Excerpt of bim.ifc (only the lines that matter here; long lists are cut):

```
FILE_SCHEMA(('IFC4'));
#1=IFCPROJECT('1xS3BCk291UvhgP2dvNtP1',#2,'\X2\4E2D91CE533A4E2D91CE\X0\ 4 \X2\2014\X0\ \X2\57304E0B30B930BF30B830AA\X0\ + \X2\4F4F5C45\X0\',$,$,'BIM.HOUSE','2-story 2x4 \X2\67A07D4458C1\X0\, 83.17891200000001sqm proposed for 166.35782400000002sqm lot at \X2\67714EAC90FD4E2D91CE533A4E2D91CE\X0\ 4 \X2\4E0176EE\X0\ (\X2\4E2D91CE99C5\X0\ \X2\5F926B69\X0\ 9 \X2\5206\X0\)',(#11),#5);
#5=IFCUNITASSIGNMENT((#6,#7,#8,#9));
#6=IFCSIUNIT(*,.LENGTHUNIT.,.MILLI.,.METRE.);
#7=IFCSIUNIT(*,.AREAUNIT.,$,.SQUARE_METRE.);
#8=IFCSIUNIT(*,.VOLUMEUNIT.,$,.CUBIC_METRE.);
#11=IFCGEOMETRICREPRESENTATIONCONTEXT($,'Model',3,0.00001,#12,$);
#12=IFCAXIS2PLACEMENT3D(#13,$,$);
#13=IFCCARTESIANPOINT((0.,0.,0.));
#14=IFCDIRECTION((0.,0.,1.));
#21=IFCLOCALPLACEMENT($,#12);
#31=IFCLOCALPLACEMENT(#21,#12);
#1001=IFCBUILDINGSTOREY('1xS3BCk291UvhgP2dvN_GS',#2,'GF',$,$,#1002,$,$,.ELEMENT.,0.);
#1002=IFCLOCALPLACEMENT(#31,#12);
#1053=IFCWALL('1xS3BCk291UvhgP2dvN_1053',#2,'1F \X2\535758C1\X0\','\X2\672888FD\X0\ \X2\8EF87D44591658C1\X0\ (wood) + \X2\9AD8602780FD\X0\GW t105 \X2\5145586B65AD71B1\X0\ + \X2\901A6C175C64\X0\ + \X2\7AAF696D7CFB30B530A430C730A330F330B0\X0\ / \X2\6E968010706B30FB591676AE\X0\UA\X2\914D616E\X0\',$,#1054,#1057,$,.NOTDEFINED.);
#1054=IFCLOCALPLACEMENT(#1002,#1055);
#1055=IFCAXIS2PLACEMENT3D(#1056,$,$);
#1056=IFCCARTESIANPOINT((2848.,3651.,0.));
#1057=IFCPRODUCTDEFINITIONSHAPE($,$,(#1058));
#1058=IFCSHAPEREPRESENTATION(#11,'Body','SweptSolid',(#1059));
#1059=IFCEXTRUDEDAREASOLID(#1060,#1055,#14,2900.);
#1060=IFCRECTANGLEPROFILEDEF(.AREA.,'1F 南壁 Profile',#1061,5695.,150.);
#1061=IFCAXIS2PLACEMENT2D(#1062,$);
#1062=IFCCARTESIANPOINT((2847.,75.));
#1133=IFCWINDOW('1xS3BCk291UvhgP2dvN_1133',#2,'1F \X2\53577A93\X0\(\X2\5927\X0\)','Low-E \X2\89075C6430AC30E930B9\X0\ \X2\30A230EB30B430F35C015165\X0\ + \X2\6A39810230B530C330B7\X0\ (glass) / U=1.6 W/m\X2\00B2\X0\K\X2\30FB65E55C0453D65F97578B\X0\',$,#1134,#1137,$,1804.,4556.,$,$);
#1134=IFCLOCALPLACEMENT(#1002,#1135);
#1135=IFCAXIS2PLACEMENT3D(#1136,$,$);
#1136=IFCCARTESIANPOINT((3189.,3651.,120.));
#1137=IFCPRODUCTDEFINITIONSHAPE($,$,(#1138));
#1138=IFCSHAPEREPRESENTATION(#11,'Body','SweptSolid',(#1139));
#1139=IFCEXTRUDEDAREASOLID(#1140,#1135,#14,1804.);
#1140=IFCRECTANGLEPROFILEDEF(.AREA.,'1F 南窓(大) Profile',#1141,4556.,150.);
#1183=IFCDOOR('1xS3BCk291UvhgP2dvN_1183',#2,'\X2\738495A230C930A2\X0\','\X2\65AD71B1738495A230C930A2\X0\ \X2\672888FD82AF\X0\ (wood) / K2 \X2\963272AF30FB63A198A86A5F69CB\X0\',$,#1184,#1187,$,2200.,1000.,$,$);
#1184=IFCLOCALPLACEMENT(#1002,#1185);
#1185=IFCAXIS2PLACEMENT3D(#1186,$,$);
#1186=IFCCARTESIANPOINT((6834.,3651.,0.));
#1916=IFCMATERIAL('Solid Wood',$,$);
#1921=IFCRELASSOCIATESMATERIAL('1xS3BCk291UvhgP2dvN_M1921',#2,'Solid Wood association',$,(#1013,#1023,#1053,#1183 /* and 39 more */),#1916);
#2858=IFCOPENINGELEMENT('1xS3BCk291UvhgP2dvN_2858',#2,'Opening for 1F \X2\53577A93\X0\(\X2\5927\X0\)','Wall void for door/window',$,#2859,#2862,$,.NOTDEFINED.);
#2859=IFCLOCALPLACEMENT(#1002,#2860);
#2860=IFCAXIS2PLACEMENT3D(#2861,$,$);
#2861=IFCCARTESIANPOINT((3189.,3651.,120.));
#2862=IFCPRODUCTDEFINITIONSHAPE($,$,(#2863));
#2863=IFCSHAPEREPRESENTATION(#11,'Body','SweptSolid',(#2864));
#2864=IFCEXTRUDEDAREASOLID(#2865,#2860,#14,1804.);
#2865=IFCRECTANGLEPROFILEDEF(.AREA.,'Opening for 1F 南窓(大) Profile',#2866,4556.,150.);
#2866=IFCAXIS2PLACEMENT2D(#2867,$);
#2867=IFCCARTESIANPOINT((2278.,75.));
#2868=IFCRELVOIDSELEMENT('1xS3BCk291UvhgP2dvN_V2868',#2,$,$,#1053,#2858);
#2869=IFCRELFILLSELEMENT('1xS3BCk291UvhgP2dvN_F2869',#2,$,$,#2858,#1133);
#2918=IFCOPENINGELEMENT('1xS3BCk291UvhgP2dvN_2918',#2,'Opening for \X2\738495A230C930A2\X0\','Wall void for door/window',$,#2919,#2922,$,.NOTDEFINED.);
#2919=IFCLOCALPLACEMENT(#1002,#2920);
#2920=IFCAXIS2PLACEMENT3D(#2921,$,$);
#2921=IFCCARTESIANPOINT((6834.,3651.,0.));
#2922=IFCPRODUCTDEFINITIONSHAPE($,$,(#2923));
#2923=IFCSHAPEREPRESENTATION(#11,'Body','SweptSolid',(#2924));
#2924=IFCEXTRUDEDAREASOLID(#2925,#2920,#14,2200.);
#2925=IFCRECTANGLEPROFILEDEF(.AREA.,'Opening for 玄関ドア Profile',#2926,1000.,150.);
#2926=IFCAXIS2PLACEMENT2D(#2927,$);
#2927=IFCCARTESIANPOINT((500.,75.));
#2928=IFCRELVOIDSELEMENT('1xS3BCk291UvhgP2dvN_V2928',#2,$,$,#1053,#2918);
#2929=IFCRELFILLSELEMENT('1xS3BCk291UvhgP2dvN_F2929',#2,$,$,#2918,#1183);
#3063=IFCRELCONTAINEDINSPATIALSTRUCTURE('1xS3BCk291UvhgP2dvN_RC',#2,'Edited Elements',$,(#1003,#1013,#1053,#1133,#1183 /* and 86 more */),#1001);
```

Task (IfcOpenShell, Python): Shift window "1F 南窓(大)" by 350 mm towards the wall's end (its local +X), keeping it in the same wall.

```python
import ifcopenshell
import ifcopenshell.api.geometry
import ifcopenshell.util.placement

model = ifcopenshell.open("bim.ifc")

window = model.by_id(1133)
opening = window.FillsVoids[0].RelatingOpeningElement
wall = opening.VoidsElements[0].RelatingBuildingElement

wall_matrix = ifcopenshell.util.placement.get_local_placement(wall.ObjectPlacement)
shift = wall_matrix[:3, 0] * 350.0
before = ifcopenshell.util.placement.get_local_placement(window.ObjectPlacement)[:3, 3].copy()

# The window is not placed relative to its opening, so move both.
for product in (opening, window):
    matrix = ifcopenshell.util.placement.get_local_placement(product.ObjectPlacement)
    matrix[:3, 3] += shift
    ifcopenshell.api.geometry.edit_object_placement(model, product=product, matrix=matrix, is_si=False)

after = ifcopenshell.util.placement.get_local_placement(window.ObjectPlacement)[:3, 3]
print("window moved by", (after - before).round(3) + 0.0)

model.write("bim_v2.ifc")
```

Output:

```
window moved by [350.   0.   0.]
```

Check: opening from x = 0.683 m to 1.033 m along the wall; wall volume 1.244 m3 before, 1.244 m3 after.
